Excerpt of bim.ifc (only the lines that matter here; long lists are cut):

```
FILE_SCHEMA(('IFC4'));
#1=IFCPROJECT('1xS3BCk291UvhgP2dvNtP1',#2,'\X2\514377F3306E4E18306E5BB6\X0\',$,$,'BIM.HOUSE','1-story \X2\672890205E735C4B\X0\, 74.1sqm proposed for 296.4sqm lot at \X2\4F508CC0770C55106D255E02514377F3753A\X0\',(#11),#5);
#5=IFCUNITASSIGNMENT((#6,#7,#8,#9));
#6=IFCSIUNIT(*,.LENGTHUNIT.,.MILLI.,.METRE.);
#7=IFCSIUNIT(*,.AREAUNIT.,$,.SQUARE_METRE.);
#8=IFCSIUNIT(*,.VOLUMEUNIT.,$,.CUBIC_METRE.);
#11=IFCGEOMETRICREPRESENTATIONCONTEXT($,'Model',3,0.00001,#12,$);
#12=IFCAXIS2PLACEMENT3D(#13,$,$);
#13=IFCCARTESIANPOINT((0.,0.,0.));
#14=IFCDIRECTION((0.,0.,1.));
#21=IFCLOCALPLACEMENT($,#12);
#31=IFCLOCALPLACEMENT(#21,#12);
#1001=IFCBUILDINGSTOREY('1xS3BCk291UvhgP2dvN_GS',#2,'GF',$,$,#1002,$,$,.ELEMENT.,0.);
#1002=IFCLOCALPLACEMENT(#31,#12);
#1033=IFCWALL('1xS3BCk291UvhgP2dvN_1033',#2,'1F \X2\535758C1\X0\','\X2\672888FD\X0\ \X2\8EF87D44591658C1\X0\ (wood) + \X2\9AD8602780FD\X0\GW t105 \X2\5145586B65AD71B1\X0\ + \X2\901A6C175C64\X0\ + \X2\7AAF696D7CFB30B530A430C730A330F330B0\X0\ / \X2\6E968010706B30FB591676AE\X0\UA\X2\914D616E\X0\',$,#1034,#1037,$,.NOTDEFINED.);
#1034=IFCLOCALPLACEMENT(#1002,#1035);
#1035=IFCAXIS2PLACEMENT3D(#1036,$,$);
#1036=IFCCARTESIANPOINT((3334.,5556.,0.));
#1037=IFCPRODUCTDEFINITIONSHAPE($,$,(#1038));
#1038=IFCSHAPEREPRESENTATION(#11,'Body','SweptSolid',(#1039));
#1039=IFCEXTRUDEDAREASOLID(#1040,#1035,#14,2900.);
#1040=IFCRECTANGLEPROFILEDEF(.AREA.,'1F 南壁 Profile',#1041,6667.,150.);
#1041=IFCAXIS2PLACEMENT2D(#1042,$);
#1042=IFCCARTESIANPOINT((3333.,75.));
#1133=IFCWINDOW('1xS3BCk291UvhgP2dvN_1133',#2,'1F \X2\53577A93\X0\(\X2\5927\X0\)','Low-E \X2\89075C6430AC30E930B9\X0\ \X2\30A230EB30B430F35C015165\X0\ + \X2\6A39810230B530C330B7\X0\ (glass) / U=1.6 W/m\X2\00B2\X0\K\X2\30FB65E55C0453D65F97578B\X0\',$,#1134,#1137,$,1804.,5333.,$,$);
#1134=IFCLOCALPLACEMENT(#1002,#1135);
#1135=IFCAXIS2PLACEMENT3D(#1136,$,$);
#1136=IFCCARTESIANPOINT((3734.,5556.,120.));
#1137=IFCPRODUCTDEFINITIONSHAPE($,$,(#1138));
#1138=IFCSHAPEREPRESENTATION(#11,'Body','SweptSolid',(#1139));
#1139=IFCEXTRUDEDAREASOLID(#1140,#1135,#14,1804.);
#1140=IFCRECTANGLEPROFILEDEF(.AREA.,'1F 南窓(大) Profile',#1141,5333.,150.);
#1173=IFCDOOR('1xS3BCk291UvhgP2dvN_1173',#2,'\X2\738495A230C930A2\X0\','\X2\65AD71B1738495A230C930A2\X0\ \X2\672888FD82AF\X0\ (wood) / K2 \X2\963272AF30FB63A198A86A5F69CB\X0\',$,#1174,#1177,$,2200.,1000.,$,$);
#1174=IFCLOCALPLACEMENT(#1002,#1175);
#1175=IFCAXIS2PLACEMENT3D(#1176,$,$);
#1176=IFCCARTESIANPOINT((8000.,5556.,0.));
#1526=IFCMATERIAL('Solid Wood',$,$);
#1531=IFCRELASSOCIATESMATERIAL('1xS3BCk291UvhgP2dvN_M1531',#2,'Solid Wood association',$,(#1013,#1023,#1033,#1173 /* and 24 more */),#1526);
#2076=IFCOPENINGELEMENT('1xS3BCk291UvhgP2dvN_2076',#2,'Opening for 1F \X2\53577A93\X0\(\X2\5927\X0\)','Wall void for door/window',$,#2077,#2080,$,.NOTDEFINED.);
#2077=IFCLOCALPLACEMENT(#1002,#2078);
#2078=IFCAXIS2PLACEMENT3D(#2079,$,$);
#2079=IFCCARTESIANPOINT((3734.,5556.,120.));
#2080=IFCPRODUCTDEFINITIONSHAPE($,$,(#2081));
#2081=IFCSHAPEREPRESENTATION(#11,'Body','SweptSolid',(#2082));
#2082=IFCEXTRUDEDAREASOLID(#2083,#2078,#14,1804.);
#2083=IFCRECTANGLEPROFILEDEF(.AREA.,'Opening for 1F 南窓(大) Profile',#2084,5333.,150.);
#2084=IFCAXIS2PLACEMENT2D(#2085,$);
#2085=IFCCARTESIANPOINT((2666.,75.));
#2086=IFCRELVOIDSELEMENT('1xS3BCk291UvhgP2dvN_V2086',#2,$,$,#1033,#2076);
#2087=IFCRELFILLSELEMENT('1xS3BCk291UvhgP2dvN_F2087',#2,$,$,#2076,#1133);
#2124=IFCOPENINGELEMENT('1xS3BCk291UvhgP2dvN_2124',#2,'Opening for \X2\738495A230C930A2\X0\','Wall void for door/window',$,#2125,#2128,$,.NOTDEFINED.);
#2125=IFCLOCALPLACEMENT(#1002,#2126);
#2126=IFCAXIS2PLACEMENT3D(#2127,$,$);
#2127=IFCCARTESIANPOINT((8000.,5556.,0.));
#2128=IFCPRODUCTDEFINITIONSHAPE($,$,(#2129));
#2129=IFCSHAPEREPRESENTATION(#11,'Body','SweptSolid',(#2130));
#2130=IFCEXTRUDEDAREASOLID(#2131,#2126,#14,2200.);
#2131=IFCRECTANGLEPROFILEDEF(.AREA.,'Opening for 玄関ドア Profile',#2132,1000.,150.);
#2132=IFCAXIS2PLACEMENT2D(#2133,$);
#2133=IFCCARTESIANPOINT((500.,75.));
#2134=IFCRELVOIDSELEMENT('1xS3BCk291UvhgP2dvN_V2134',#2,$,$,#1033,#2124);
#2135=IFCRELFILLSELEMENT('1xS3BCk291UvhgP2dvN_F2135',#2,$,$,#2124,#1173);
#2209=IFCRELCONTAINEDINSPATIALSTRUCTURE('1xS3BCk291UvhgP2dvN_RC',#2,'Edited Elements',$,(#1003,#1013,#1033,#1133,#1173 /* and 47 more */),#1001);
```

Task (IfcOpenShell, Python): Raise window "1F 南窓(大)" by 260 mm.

```python
import numpy as np
import ifcopenshell
import ifcopenshell.api.geometry
import ifcopenshell.util.placement
import ifcopenshell.util.unit

model = ifcopenshell.open("bim.ifc")
unit_scale = ifcopenshell.util.unit.calculate_unit_scale(model)

window = model.by_guid("1xS3BCk291UvhgP2dvN_1133")
opening = window.FillsVoids[0].RelatingOpeningElement
dz = 0.26 / unit_scale

shift = np.array([0.0, 0.0, dz])
# The window is not placed relative to its opening, so move both.
for product in (opening, window):
    matrix = ifcopenshell.util.placement.get_local_placement(product.ObjectPlacement)
    matrix[:3, 3] += shift
    ifcopenshell.api.geometry.edit_object_placement(model, product=product, matrix=matrix, is_si=False)

print(f"moved by {dz * unit_scale:+.3f} m")

model.write("bim-out.ifc")
```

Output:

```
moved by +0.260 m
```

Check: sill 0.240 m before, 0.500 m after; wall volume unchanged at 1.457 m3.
